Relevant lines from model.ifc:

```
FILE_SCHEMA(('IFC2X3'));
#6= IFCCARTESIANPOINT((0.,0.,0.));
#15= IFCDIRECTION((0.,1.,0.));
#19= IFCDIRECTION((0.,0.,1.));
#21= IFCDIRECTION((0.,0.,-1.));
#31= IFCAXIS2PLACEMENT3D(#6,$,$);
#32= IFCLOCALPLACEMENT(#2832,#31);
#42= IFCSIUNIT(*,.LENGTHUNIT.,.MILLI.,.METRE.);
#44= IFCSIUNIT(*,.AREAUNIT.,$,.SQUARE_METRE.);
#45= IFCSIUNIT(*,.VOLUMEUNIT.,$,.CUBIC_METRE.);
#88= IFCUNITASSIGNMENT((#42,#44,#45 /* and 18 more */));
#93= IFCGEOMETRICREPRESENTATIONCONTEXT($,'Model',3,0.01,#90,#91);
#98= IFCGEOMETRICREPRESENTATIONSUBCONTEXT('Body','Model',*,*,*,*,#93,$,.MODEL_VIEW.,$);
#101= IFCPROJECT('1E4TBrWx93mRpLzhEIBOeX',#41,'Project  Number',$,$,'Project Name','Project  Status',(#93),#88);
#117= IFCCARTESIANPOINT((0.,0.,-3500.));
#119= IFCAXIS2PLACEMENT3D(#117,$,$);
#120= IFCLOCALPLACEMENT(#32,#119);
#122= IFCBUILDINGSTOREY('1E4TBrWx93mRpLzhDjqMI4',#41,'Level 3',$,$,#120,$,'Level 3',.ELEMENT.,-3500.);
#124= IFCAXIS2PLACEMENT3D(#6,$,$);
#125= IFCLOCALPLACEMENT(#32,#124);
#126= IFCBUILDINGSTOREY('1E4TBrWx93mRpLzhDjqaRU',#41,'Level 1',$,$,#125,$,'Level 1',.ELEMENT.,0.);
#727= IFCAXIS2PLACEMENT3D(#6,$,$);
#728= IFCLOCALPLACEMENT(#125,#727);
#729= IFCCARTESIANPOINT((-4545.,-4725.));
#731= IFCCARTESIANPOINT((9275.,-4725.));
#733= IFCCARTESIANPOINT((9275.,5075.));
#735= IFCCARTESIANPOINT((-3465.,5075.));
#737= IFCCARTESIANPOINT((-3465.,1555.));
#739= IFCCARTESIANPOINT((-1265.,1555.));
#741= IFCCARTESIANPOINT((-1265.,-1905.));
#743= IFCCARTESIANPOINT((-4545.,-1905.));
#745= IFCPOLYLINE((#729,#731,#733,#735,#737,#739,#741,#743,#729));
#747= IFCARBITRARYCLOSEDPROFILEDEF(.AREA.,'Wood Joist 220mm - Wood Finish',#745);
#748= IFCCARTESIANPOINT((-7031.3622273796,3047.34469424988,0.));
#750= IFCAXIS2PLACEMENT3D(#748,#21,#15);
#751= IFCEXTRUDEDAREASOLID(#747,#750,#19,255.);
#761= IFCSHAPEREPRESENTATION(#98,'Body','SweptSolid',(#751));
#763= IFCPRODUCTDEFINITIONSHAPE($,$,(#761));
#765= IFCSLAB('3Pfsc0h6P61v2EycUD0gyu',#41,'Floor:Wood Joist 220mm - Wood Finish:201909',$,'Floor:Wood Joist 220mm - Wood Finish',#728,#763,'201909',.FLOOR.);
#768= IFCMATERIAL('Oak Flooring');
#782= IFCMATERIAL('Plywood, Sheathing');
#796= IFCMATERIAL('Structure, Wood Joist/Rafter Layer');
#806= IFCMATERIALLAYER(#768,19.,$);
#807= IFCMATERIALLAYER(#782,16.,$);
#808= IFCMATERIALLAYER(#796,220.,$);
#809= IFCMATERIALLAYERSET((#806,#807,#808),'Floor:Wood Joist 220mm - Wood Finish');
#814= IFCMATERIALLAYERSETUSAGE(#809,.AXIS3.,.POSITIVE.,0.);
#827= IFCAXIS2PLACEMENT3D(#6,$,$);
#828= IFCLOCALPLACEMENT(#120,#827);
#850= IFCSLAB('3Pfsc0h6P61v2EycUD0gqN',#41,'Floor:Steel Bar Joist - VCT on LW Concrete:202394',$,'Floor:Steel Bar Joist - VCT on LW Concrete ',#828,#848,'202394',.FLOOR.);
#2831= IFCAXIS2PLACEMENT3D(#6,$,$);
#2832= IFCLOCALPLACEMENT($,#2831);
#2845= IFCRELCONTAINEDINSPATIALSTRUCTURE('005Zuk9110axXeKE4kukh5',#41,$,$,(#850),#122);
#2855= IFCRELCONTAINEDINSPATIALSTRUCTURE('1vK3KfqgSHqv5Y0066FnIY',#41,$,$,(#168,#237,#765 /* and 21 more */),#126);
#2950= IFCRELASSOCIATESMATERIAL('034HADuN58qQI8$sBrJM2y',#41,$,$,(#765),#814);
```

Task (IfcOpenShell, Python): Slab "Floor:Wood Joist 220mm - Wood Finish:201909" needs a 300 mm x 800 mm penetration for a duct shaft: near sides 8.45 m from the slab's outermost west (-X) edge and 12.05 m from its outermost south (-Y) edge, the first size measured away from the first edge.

```python
import numpy as np
import ifcopenshell
import ifcopenshell.api.feature
import ifcopenshell.api.geometry
import ifcopenshell.api.root
import ifcopenshell.geom
import ifcopenshell.util.placement
import ifcopenshell.util.representation
import ifcopenshell.util.shape
import ifcopenshell.util.unit

model = ifcopenshell.open("model.ifc")
unit_scale = ifcopenshell.util.unit.calculate_unit_scale(model)
settings = ifcopenshell.geom.settings()


def volume(element):
    """Net volume in cubic metres, openings subtracted."""
    shape = ifcopenshell.geom.create_shape(settings, element)
    return ifcopenshell.util.shape.get_volume(shape.geometry)


slab = model.by_guid("3Pfsc0h6P61v2EycUD0gyu")
before = volume(slab)

# Extent in the slab's own axes, in metres. The edges named are its -X and -Y sides.
slab_shape = ifcopenshell.geom.create_shape(settings, slab)
vertices = ifcopenshell.util.shape.get_vertices(slab_shape.geometry)
x_min, y_min, bottom = vertices.min(axis=0)
top = vertices[:, 2].max()

opening = ifcopenshell.api.root.create_entity(model, ifc_class="IfcOpeningElement", name="Duct shaft opening")
context = ifcopenshell.util.representation.get_context(model, "Model", "Body", "MODEL_VIEW")
width, depth = 0.3, 0.8
outline = [(0.0, 0.0), (width, 0.0), (width, depth), (0.0, depth), (0.0, 0.0)]
# Overshoot both faces by 50 mm so the cut is clean.
shape = ifcopenshell.api.geometry.add_slab_representation(
    model, context=context, depth=top - bottom + 0.1, polyline=outline
)
ifcopenshell.api.geometry.assign_representation(model, product=opening, representation=shape)

matrix = ifcopenshell.util.placement.get_local_placement(slab.ObjectPlacement)
matrix[:, 3] = matrix @ np.append(np.array([x_min + 8.45, y_min + 12.05, bottom - 0.05]) / unit_scale, 1.0)
ifcopenshell.api.geometry.edit_object_placement(model, product=opening, matrix=matrix, is_si=False)
ifcopenshell.api.feature.add_feature(model, feature=opening, element=slab)

after = volume(slab)

print(f"slab volume {before:.3f} -> {after:.3f} m3")

model.write("model_rev.ifc")
```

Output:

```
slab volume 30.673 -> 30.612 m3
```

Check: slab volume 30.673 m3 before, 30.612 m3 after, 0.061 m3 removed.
